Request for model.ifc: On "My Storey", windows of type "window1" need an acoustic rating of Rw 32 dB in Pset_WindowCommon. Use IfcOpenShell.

First a look at what the model holds.

```python
import ifcopenshell
import ifcopenshell.util.element

model = ifcopenshell.open("model.ifc")
print(model.schema)
storey = next(s for s in model.by_type("IfcBuildingStorey") if s.Name == "My Storey")
windows = [e for e in ifcopenshell.util.element.get_decomposition(storey) if e.is_a("IfcWindow")]
seen = {}
for e in windows:
    element_type = ifcopenshell.util.element.get_type(e)
    key = (element_type.Name if element_type != e and element_type else None, ifcopenshell.util.element.get_pset(e, "Pset_WindowCommon", "AcousticRating"))
    seen[key] = seen.get(key, 0) + 1
for (name, value), count in sorted(seen.items(), key=str):
    print(count, "x", name, "|", value)
```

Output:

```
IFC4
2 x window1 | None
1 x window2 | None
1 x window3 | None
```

```python
import ifcopenshell
import ifcopenshell.api.pset
import ifcopenshell.util.element

model = ifcopenshell.open("model.ifc")

storey = next(s for s in model.by_type("IfcBuildingStorey") if s.Name == "My Storey")
windows = [e for e in ifcopenshell.util.element.get_decomposition(storey) if e.is_a("IfcWindow")]

count = 0
for e in windows:
    element_type = ifcopenshell.util.element.get_type(e)
    if element_type in (None, e) or element_type.Name != "window1":
        continue
    # add_pset returns the element's existing set when there is one.
    pset = ifcopenshell.api.pset.add_pset(model, product=e, name="Pset_WindowCommon")
    ifcopenshell.api.pset.edit_pset(model, pset=pset, properties={"AcousticRating": "Rw 32 dB"})
    count += 1

print(count, "windows updated")

model.write("model_edited.ifc")
```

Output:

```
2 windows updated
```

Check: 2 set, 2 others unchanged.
